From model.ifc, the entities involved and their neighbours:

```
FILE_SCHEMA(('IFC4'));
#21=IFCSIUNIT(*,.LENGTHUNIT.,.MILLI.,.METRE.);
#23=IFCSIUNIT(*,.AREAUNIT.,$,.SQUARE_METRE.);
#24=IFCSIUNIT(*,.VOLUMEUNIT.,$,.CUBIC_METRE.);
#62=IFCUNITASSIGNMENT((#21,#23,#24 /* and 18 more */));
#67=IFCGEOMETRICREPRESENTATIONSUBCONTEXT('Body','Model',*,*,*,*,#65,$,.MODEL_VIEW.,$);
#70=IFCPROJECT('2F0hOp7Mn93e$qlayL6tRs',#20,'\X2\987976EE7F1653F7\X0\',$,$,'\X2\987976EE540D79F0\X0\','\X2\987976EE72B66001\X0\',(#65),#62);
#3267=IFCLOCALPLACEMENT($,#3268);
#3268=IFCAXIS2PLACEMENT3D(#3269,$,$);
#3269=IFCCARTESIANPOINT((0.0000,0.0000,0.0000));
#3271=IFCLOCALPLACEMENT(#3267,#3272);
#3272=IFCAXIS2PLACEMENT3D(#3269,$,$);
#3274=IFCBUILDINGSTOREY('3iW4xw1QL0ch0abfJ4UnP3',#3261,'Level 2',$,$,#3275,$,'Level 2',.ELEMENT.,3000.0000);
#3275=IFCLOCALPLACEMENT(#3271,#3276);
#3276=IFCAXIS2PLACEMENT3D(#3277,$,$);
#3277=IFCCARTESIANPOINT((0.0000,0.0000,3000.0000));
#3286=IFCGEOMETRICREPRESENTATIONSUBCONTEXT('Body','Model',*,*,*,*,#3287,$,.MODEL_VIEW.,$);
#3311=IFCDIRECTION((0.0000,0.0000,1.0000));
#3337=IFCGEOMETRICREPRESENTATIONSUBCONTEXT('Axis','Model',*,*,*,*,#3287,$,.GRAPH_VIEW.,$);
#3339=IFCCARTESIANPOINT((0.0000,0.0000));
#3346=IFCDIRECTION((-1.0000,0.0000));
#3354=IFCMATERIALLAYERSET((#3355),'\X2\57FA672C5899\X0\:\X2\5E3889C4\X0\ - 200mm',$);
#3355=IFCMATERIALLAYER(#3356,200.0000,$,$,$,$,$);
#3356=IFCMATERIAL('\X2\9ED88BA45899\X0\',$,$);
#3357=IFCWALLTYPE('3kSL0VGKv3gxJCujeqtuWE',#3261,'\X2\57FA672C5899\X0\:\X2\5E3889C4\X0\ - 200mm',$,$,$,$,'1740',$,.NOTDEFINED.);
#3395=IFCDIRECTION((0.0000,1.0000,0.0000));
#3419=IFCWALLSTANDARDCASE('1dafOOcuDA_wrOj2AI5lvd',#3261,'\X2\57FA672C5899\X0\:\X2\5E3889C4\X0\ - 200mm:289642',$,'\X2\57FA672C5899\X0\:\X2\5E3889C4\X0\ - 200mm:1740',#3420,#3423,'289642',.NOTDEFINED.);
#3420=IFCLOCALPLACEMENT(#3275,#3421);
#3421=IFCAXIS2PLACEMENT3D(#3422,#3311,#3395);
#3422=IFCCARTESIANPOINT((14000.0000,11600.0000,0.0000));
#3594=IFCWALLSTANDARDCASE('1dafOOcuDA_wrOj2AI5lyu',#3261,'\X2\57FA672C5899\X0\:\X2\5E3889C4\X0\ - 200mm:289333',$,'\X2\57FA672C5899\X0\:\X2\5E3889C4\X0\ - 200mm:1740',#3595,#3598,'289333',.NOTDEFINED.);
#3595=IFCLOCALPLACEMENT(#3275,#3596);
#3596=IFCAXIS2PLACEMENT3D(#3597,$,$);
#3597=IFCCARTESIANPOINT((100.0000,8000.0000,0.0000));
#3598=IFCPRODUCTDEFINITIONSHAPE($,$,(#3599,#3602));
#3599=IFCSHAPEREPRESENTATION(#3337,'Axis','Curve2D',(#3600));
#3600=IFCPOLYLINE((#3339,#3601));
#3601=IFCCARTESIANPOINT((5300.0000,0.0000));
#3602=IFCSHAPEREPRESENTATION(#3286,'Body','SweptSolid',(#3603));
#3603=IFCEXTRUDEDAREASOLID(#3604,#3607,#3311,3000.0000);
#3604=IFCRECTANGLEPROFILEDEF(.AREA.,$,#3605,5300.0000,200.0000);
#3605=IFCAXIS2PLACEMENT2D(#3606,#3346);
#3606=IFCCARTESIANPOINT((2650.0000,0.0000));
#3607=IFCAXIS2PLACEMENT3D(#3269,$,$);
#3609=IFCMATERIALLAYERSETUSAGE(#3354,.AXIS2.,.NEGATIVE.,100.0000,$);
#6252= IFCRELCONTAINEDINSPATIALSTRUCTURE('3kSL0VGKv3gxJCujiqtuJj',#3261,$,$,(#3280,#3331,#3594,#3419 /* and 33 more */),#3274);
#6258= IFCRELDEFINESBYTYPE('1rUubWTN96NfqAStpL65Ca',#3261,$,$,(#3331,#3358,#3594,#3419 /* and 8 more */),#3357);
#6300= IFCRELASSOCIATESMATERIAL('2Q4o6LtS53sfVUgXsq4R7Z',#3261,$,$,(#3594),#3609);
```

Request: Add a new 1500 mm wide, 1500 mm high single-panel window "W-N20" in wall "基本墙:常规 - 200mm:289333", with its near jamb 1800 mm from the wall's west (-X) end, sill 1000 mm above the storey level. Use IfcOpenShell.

```python
import numpy as np
import ifcopenshell
import ifcopenshell.api.feature
import ifcopenshell.api.geometry
import ifcopenshell.api.root
import ifcopenshell.api.spatial
import ifcopenshell.geom
import ifcopenshell.util.element
import ifcopenshell.util.placement
import ifcopenshell.util.representation
import ifcopenshell.util.shape
import ifcopenshell.util.unit

model = ifcopenshell.open("model.ifc")
unit_scale = ifcopenshell.util.unit.calculate_unit_scale(model)
settings = ifcopenshell.geom.settings()


def volume(element):
    """Net volume in cubic metres, openings subtracted."""
    shape = ifcopenshell.geom.create_shape(settings, element)
    return ifcopenshell.util.shape.get_volume(shape.geometry)


wall = model.by_guid("1dafOOcuDA_wrOj2AI5lyu")
storey = ifcopenshell.util.element.get_container(wall, ifc_class="IfcBuildingStorey")
context = ifcopenshell.util.representation.get_context(model, "Model", "Body", "MODEL_VIEW")
before = volume(wall)

width, height, from_end, sill = 1.5, 1.5, 1.8, 1  # metres

# The wall runs along its own X axis, and the end named is its -X end.
wall_shape = ifcopenshell.geom.create_shape(settings, wall)
x, y, z = ifcopenshell.util.shape.get_vertices(wall_shape.geometry).T
start = x.min() + from_end
face, thickness = float(y.min()), float(y.max() - y.min())
wall_matrix = ifcopenshell.util.placement.get_local_placement(wall.ObjectPlacement)
level = ifcopenshell.util.placement.get_local_placement(storey.ObjectPlacement)[2, 3]


def in_wall(x, y):
    """Placement at x, y metres in the wall's axes, at sill height."""
    matrix = wall_matrix.copy()
    matrix[:, 3] = wall_matrix @ np.array([x / unit_scale, y / unit_scale, 0.0, 1.0])
    matrix[2, 3] = level + sill / unit_scale
    return matrix


# Opening: a box that overshoots both wall faces by 50 mm.
opening = ifcopenshell.api.root.create_entity(model, ifc_class="IfcOpeningElement", predefined_type="OPENING")
box = ifcopenshell.api.geometry.add_wall_representation(
    model, context=context, length=width, height=height, thickness=thickness + 0.1
)
ifcopenshell.api.geometry.assign_representation(model, product=opening, representation=box)
ifcopenshell.api.geometry.edit_object_placement(model, product=opening, matrix=in_wall(start, face - 0.05), is_si=False)
ifcopenshell.api.feature.add_feature(model, feature=opening, element=wall)

window = ifcopenshell.api.root.create_entity(model, ifc_class="IfcWindow", name="W-N20", predefined_type="WINDOW")
window.OverallWidth, window.OverallHeight = width / unit_scale, height / unit_scale
window.PartitioningType = "SINGLE_PANEL"
body = ifcopenshell.api.geometry.add_window_representation(
    model,
    context=context,
    overall_width=window.OverallWidth,
    overall_height=window.OverallHeight,
    partition_type="SINGLE_PANEL",
)
ifcopenshell.api.geometry.assign_representation(model, product=window, representation=body)
ifcopenshell.api.spatial.assign_container(model, products=[window], relating_structure=storey)
ifcopenshell.api.feature.add_filling(model, opening=opening, element=window)

# Centre the window in the wall's thickness.
ifcopenshell.api.geometry.edit_object_placement(model, product=window, matrix=in_wall(start, face), is_si=False)
window_shape = ifcopenshell.geom.create_shape(settings, window)
depth = ifcopenshell.util.shape.get_vertices(window_shape.geometry)[:, 1]
offset = face + thickness / 2 - (depth.min() + depth.max()) / 2
ifcopenshell.api.geometry.edit_object_placement(model, product=window, matrix=in_wall(start, offset), is_si=False)

after = volume(wall)

print(f"wall volume {before:.3f} -> {after:.3f} m3")

model.write("model-out.ifc")
```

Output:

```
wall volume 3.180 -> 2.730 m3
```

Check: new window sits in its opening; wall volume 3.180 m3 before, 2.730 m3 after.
